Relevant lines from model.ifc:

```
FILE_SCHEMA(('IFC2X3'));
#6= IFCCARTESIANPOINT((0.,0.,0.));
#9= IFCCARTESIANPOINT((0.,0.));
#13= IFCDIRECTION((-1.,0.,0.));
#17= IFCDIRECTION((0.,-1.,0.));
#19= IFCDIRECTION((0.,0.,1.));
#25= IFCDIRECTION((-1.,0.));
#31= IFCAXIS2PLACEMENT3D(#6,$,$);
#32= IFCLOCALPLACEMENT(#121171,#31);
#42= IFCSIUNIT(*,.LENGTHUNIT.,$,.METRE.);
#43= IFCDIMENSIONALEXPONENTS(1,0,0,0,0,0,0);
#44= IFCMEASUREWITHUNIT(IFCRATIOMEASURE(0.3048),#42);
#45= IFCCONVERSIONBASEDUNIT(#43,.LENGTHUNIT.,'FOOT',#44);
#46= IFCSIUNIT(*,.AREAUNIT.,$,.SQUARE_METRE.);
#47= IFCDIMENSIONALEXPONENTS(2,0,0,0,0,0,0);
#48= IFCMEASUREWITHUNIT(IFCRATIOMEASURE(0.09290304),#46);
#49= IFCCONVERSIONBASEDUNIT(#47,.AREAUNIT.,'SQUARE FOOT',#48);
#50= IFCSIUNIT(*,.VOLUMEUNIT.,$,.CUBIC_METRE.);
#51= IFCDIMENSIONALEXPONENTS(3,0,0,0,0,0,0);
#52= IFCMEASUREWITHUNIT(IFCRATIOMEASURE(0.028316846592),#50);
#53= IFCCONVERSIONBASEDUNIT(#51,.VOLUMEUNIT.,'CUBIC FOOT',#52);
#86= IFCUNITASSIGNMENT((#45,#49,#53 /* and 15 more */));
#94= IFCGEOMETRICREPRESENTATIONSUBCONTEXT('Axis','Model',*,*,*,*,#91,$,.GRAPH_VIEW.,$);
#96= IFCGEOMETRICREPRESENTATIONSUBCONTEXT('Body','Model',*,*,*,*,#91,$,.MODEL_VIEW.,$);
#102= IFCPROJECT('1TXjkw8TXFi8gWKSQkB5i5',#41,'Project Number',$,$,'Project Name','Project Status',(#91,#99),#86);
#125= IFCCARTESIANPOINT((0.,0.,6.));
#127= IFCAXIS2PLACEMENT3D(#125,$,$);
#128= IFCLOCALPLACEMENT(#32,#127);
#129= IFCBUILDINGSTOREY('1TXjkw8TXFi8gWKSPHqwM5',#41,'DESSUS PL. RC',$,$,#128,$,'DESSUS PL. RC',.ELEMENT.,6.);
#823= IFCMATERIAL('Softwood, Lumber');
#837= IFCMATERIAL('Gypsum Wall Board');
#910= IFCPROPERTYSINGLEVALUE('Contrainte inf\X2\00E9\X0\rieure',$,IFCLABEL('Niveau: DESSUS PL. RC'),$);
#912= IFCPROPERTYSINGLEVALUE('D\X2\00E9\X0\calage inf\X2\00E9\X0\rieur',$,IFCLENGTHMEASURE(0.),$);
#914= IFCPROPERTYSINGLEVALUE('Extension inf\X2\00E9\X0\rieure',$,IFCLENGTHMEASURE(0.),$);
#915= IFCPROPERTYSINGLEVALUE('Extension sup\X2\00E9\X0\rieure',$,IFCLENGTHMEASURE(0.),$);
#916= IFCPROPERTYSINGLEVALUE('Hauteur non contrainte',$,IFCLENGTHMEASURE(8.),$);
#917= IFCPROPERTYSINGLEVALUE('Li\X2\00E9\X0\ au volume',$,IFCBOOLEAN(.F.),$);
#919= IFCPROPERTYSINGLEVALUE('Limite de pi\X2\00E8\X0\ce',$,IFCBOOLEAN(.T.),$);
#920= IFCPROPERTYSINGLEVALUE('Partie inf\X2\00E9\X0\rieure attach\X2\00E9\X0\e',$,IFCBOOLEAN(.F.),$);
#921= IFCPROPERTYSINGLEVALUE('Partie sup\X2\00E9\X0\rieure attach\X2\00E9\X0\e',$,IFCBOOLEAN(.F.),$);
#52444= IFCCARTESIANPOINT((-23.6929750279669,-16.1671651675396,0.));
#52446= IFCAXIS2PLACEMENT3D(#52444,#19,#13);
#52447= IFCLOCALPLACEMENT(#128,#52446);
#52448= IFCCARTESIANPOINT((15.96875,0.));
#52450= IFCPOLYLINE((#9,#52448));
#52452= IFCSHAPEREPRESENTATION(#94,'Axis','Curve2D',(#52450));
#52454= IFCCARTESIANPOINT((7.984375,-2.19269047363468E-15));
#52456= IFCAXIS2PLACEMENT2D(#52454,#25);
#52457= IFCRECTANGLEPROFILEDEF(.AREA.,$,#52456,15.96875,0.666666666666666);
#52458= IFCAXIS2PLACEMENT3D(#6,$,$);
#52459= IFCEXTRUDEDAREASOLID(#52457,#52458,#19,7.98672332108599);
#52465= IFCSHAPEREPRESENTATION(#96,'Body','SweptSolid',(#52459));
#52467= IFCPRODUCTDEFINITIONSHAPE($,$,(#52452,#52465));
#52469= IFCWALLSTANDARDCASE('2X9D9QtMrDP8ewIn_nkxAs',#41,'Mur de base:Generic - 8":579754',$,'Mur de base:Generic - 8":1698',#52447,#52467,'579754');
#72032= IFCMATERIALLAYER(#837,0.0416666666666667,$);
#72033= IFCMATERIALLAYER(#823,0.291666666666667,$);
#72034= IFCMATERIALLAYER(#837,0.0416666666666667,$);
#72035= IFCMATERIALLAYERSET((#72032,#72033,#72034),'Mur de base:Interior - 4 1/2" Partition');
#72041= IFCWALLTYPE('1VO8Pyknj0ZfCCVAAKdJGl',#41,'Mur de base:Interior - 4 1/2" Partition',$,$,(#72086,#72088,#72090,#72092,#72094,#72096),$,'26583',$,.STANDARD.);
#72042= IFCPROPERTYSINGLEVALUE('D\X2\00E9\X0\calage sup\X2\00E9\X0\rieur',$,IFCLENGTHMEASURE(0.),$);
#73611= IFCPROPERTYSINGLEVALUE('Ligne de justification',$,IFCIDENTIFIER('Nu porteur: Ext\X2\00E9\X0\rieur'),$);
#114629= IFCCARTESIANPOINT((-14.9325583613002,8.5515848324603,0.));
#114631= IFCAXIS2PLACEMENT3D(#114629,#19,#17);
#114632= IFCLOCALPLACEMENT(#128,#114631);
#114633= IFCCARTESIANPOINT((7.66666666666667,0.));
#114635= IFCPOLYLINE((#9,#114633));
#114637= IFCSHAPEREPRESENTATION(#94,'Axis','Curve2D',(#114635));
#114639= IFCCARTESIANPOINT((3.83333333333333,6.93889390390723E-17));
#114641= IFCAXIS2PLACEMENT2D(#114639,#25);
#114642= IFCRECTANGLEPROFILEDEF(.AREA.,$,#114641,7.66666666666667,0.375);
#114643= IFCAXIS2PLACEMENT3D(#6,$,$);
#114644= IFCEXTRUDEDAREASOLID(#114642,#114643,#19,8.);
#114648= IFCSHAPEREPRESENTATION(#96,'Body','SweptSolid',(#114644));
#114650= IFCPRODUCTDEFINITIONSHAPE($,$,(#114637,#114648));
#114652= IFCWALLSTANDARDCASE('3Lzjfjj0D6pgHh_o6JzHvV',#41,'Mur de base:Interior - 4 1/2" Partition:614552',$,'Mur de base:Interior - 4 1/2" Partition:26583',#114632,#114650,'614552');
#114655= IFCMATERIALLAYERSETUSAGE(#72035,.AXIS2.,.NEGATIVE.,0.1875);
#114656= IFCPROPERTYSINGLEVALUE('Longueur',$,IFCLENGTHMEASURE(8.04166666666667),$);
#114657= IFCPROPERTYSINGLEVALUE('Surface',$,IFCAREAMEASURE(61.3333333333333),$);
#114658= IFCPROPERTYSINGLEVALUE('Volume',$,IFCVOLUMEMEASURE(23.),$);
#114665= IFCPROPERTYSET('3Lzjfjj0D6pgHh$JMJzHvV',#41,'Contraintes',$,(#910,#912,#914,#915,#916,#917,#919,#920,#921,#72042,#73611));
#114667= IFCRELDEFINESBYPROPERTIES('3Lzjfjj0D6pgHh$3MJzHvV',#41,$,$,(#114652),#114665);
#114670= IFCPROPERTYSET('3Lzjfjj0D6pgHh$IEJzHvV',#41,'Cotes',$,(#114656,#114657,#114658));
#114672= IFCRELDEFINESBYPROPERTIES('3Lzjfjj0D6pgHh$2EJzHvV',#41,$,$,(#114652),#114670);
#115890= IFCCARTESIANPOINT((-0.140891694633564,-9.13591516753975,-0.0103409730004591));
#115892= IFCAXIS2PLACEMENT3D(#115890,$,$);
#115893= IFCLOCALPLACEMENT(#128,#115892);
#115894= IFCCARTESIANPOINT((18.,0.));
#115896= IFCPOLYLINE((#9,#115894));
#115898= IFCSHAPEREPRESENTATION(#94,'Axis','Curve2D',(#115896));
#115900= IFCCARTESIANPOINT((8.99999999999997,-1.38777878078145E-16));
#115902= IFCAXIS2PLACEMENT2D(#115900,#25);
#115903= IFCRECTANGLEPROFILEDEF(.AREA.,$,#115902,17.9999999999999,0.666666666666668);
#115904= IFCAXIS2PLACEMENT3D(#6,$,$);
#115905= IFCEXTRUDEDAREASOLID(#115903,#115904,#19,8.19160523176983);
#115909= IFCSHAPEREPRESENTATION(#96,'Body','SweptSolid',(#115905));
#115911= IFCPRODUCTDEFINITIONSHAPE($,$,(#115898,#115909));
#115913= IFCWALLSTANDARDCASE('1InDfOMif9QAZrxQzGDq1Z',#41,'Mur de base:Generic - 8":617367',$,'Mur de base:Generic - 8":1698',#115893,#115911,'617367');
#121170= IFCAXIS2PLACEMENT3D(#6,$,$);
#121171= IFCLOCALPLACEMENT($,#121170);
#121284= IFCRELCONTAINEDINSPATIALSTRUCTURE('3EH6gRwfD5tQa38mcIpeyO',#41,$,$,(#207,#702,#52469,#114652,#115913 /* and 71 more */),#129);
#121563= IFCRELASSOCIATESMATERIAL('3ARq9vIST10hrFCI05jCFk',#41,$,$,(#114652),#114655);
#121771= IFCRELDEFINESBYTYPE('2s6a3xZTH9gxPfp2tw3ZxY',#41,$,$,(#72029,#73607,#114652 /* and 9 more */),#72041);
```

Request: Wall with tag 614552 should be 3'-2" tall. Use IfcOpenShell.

```python
import ifcopenshell
import ifcopenshell.api.pset
import ifcopenshell.geom
import ifcopenshell.util.element
import ifcopenshell.util.representation
import ifcopenshell.util.shape
import ifcopenshell.util.unit

model = ifcopenshell.open("model.ifc")
unit_scale = ifcopenshell.util.unit.calculate_unit_scale(model)
area_scale = ifcopenshell.util.unit.calculate_unit_scale(model, "AREAUNIT")
volume_scale = ifcopenshell.util.unit.calculate_unit_scale(model, "VOLUMEUNIT")
settings = ifcopenshell.geom.settings()


def volume(element):
    """Net volume in cubic metres, openings subtracted."""
    shape = ifcopenshell.geom.create_shape(settings, element)
    return ifcopenshell.util.shape.get_volume(shape.geometry)


wall = model.by_guid("3Lzjfjj0D6pgHh_o6JzHvV")
before = volume(wall)

body = ifcopenshell.util.representation.get_representation(wall, "Model", "Body")
solid = body.Items[0]
old_height = solid.Depth
solid.Depth = 38 * 0.0254 / unit_scale
after = volume(wall)
thickness = 0.1143  # wall thickness in metres

# Update the stored height, areas and volumes.
pset = model.by_id(ifcopenshell.util.element.get_pset(wall, "Contraintes", should_inherit=False)["id"])
ifcopenshell.api.pset.edit_pset(model, pset=pset, properties={
    "Hauteur non contrainte": model.create_entity("IfcLengthMeasure", solid.Depth),
})
pset = model.by_id(ifcopenshell.util.element.get_pset(wall, "Cotes", should_inherit=False)["id"])
ifcopenshell.api.pset.edit_pset(model, pset=pset, properties={
    "Surface": model.create_entity("IfcAreaMeasure", after / thickness / area_scale),
    "Volume": model.create_entity("IfcVolumeMeasure", after / volume_scale),
})

print(f"height {old_height:g} -> {solid.Depth:g}, volume {before:.3f} -> {after:.3f} m3")

model.write("model_v2.ifc")
```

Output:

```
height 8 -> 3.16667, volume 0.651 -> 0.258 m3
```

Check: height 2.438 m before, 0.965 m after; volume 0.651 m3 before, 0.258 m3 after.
